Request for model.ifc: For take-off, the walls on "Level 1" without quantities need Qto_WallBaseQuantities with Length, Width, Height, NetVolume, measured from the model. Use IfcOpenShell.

First a look at what the model holds.

```python
import ifcopenshell
import ifcopenshell.util.element
import ifcopenshell.util.unit

model = ifcopenshell.open("model.ifc")
print(model.schema)
for unit_type in ("LENGTHUNIT", "AREAUNIT", "VOLUMEUNIT"):
    print(unit_type, ifcopenshell.util.unit.calculate_unit_scale(model, unit_type))
storey = next(s for s in model.by_type("IfcBuildingStorey") if s.Name == "Level 1")
walls = [e for e in ifcopenshell.util.element.get_decomposition(storey) if e.is_a("IfcWall")]
for e in sorted(walls, key=lambda e: e.id()):
    print(e.id(), e.is_a(), e.Name, list(ifcopenshell.util.element.get_psets(e, qtos_only=True)), sep=" | ")
```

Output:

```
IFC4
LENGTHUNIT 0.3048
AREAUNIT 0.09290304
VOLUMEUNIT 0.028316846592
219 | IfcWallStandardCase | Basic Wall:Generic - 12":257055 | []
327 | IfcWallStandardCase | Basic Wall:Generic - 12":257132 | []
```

```python
import ifcopenshell
import ifcopenshell.api.pset
import ifcopenshell.geom
import ifcopenshell.util.element
import ifcopenshell.util.shape
import ifcopenshell.util.unit

model = ifcopenshell.open("model.ifc")
unit_scale = ifcopenshell.util.unit.calculate_unit_scale(model)
volume_scale = ifcopenshell.util.unit.calculate_unit_scale(model, "VOLUMEUNIT")
settings = ifcopenshell.geom.settings()

storey = next(s for s in model.by_type("IfcBuildingStorey") if s.Name == "Level 1")
walls = [e for e in ifcopenshell.util.element.get_decomposition(storey) if e.is_a("IfcWall")]

for e in sorted(walls, key=lambda e: e.id()):
    if ifcopenshell.util.element.get_psets(e, qtos_only=True, should_inherit=False):
        continue
    # Geometry comes back in metres, in the element's own axes.
    shape = ifcopenshell.geom.create_shape(settings, e)
    values = {
        "Length": ifcopenshell.util.shape.get_x(shape.geometry) / unit_scale,
        "Width": ifcopenshell.util.shape.get_y(shape.geometry) / unit_scale,
        "Height": ifcopenshell.util.shape.get_z(shape.geometry) / unit_scale,
        "NetVolume": ifcopenshell.util.shape.get_volume(shape.geometry) / volume_scale,
    }
    qto = ifcopenshell.api.pset.add_qto(model, product=e, name="Qto_WallBaseQuantities")
    ifcopenshell.api.pset.edit_qto(model, qto=qto, properties=values)
    print(e.id(), {k: round(v, 3) for k, v in values.items()})

model.write("model_rev.ifc")
```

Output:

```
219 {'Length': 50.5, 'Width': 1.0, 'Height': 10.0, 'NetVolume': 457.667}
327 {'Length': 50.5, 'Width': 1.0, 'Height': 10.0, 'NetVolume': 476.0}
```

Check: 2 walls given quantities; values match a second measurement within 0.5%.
